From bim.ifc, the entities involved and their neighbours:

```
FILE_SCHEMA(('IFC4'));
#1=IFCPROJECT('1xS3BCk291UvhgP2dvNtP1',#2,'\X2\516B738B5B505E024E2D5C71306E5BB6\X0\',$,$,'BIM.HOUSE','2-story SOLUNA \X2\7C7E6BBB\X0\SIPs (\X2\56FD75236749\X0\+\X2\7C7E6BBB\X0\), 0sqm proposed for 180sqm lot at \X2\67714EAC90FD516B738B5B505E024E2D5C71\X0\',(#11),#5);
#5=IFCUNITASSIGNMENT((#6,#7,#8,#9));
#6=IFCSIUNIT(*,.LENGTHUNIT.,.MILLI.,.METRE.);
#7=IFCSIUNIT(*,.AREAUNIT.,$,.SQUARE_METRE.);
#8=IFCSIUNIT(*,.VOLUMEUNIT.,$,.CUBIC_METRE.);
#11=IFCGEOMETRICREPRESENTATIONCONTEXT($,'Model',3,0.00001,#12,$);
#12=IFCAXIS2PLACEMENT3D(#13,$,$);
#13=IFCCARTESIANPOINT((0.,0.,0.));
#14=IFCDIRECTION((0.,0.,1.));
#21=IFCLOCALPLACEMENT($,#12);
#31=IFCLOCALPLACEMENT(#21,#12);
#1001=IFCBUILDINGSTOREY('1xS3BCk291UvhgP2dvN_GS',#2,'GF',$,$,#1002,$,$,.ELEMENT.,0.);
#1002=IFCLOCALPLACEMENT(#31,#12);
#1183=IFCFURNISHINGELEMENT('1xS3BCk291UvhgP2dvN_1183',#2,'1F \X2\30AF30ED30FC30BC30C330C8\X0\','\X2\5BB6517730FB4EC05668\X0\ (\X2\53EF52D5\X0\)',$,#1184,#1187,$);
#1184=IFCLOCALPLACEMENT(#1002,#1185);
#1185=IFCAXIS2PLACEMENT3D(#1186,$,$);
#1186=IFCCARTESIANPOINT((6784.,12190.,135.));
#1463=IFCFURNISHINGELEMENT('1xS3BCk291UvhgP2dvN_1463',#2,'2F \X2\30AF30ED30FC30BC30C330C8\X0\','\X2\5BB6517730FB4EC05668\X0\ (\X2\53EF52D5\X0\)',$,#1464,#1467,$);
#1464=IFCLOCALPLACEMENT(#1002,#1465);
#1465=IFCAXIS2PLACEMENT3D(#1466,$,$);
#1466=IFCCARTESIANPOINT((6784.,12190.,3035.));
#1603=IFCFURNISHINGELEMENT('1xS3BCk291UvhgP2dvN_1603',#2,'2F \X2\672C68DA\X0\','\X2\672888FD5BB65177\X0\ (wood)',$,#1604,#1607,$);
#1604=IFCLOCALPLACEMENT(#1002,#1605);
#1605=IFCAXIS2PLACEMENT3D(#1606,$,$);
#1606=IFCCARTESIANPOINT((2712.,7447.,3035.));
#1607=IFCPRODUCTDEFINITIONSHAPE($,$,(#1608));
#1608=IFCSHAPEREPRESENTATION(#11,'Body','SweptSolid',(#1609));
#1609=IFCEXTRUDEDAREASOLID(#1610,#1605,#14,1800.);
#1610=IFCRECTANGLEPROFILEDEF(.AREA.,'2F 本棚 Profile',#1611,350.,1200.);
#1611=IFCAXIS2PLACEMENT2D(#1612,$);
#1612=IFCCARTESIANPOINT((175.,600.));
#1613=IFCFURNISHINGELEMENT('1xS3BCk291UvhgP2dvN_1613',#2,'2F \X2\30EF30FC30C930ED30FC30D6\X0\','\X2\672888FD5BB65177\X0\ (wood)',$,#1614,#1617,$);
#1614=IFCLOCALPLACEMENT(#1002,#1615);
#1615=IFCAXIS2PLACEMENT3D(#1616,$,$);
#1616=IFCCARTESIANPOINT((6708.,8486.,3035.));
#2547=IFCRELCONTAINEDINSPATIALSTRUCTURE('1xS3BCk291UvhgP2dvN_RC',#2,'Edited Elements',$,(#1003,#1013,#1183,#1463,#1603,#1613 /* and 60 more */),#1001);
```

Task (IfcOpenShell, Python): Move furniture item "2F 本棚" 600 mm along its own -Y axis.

```python
import ifcopenshell
import ifcopenshell.api.geometry
import ifcopenshell.util.placement
import ifcopenshell.util.unit

model = ifcopenshell.open("bim.ifc")
unit_scale = ifcopenshell.util.unit.calculate_unit_scale(model)

item = model.by_guid("1xS3BCk291UvhgP2dvN_1603")
matrix = ifcopenshell.util.placement.get_local_placement(item.ObjectPlacement)
matrix[:3, 3] -= matrix[:3, 1] * 0.6 / unit_scale
ifcopenshell.api.geometry.edit_object_placement(model, product=item, matrix=matrix, is_si=False)

print(ifcopenshell.util.placement.get_local_placement(item.ObjectPlacement).round(3) + 0.0)

model.write("bim_rev.ifc")
```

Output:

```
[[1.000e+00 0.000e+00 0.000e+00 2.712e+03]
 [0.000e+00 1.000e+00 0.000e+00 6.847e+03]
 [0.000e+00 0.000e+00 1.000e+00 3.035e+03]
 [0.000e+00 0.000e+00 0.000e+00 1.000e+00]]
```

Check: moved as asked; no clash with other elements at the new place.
